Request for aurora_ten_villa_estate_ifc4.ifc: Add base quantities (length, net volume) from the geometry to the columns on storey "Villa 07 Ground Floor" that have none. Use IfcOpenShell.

First a look at what the model holds.

```python
import ifcopenshell
import ifcopenshell.util.element
import ifcopenshell.util.unit

model = ifcopenshell.open("aurora_ten_villa_estate_ifc4.ifc")
print(model.schema)
for unit_type in ("LENGTHUNIT", "AREAUNIT", "VOLUMEUNIT"):
    print(unit_type, ifcopenshell.util.unit.calculate_unit_scale(model, unit_type))
storey = next(s for s in model.by_type("IfcBuildingStorey") if s.Name == "Villa 07 Ground Floor")
columns = [e for e in ifcopenshell.util.element.get_decomposition(storey) if e.is_a("IfcColumn")]
for e in sorted(columns, key=lambda e: e.id()):
    print(e.id(), e.is_a(), e.Name, list(ifcopenshell.util.element.get_psets(e, qtos_only=True)), sep=" | ")
```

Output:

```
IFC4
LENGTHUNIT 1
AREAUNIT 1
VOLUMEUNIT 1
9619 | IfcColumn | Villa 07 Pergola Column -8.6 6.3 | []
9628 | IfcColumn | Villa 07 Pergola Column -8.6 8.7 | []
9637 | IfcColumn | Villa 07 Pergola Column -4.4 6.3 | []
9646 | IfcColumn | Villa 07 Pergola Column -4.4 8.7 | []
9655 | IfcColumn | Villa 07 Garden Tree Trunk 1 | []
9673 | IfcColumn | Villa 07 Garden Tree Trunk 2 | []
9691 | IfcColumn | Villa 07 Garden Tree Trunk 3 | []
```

```python
import ifcopenshell
import ifcopenshell.api.pset
import ifcopenshell.geom
import ifcopenshell.util.element
import ifcopenshell.util.shape
import ifcopenshell.util.unit

model = ifcopenshell.open("aurora_ten_villa_estate_ifc4.ifc")
unit_scale = ifcopenshell.util.unit.calculate_unit_scale(model)
volume_scale = ifcopenshell.util.unit.calculate_unit_scale(model, "VOLUMEUNIT")
settings = ifcopenshell.geom.settings()

storey = next(s for s in model.by_type("IfcBuildingStorey") if s.Name == "Villa 07 Ground Floor")
columns = [e for e in ifcopenshell.util.element.get_decomposition(storey) if e.is_a("IfcColumn")]

for e in sorted(columns, key=lambda e: e.id()):
    if ifcopenshell.util.element.get_psets(e, qtos_only=True, should_inherit=False):
        continue
    # Geometry comes back in metres, in the element's own axes.
    shape = ifcopenshell.geom.create_shape(settings, e)
    values = {
        "Length": ifcopenshell.util.shape.get_z(shape.geometry) / unit_scale,
        "NetVolume": ifcopenshell.util.shape.get_volume(shape.geometry) / volume_scale,
    }
    qto = ifcopenshell.api.pset.add_qto(model, product=e, name="Qto_ColumnBaseQuantities")
    ifcopenshell.api.pset.edit_qto(model, qto=qto, properties=values)
    print(e.id(), {k: round(v, 3) for k, v in values.items()})

model.write("aurora_ten_villa_estate_ifc4_rev.ifc")
```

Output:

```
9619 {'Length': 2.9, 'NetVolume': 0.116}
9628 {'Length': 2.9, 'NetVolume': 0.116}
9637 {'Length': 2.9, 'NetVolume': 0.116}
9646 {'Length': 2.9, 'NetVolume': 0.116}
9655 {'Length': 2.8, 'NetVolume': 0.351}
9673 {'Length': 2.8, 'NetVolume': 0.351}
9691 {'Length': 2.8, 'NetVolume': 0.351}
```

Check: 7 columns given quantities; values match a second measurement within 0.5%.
